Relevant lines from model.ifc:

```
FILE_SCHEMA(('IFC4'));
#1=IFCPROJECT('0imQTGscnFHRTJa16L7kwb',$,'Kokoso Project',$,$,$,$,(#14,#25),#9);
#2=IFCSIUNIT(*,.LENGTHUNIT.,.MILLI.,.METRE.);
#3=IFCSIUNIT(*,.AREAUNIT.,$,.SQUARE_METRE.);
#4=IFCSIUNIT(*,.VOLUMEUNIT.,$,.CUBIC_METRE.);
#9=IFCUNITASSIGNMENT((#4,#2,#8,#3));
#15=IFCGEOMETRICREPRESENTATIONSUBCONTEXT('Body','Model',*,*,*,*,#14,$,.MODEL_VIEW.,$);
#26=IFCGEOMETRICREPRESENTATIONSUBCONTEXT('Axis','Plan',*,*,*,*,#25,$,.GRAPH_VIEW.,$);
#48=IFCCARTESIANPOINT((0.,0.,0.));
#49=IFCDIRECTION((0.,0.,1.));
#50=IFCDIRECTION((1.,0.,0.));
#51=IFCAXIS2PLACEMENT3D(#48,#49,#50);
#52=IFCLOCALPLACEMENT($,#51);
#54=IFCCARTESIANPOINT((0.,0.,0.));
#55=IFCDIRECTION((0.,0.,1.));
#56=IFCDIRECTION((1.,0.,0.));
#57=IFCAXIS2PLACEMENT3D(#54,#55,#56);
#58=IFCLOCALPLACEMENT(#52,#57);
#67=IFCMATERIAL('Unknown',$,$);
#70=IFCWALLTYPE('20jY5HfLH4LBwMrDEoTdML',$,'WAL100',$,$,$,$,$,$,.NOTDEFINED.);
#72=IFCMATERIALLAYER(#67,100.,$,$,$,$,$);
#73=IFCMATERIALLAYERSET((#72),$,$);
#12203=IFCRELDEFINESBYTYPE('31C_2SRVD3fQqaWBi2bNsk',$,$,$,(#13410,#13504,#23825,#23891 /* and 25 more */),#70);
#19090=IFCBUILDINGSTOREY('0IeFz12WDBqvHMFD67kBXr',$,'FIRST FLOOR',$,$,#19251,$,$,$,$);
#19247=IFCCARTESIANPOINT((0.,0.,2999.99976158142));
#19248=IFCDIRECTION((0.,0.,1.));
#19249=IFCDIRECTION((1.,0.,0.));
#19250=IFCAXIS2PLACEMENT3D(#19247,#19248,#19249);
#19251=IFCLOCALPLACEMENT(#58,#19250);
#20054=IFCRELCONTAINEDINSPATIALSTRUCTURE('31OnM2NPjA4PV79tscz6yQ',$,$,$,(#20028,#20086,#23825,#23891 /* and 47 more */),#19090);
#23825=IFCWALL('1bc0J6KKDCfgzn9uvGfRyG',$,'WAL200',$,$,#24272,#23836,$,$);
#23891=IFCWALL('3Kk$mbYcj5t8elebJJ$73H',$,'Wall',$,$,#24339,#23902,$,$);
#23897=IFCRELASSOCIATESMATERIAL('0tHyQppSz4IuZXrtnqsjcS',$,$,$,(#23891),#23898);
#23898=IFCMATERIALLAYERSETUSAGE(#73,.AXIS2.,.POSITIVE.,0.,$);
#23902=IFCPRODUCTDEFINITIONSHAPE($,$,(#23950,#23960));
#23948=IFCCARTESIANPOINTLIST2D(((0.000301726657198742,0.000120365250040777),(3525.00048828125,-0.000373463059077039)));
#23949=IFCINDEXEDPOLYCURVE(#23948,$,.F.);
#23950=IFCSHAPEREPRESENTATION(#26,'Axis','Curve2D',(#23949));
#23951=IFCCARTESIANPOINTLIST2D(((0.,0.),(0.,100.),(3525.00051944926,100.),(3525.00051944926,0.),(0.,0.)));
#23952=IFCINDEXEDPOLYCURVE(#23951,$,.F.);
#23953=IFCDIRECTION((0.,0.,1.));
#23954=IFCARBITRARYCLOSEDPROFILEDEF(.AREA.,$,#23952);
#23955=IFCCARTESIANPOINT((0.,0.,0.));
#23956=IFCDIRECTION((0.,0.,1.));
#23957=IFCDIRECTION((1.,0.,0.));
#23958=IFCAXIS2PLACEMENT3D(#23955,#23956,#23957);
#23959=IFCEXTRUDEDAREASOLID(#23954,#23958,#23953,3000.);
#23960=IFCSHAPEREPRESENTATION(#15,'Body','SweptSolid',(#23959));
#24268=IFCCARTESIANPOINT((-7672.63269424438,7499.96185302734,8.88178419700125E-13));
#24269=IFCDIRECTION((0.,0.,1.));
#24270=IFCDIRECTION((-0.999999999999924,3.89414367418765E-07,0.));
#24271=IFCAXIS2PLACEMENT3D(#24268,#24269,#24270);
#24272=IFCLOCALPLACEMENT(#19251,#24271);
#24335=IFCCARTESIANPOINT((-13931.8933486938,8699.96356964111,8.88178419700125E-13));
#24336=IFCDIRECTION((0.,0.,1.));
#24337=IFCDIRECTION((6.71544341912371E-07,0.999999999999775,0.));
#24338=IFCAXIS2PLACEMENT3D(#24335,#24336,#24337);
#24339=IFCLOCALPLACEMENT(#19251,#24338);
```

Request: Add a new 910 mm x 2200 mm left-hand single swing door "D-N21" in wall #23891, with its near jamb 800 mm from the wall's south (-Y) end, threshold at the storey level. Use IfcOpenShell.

```python
import numpy as np
import ifcopenshell
import ifcopenshell.api.feature
import ifcopenshell.api.geometry
import ifcopenshell.api.root
import ifcopenshell.api.spatial
import ifcopenshell.geom
import ifcopenshell.util.element
import ifcopenshell.util.placement
import ifcopenshell.util.representation
import ifcopenshell.util.shape
import ifcopenshell.util.unit

model = ifcopenshell.open("model.ifc")
unit_scale = ifcopenshell.util.unit.calculate_unit_scale(model)
settings = ifcopenshell.geom.settings()


def volume(element):
    """Net volume in cubic metres, openings subtracted."""
    shape = ifcopenshell.geom.create_shape(settings, element)
    return ifcopenshell.util.shape.get_volume(shape.geometry)


wall = model.by_guid("3Kk$mbYcj5t8elebJJ$73H")
storey = ifcopenshell.util.element.get_container(wall, ifc_class="IfcBuildingStorey")
context = ifcopenshell.util.representation.get_context(model, "Model", "Body", "MODEL_VIEW")
before = volume(wall)

width, height, from_end, sill = 0.91, 2.2, 0.8, 0.0  # metres

# The wall runs along its own X axis, and the end named is its -X end.
wall_shape = ifcopenshell.geom.create_shape(settings, wall)
x, y, z = ifcopenshell.util.shape.get_vertices(wall_shape.geometry).T
start = x.min() + from_end
face, thickness = float(y.min()), float(y.max() - y.min())
wall_matrix = ifcopenshell.util.placement.get_local_placement(wall.ObjectPlacement)
level = ifcopenshell.util.placement.get_local_placement(storey.ObjectPlacement)[2, 3]


def in_wall(x, y):
    """Placement at x, y metres in the wall's axes, at sill height."""
    matrix = wall_matrix.copy()
    matrix[:, 3] = wall_matrix @ np.array([x / unit_scale, y / unit_scale, 0.0, 1.0])
    matrix[2, 3] = level + sill / unit_scale
    return matrix


# Opening: a box that overshoots both wall faces by 50 mm.
opening = ifcopenshell.api.root.create_entity(model, ifc_class="IfcOpeningElement", predefined_type="OPENING")
box = ifcopenshell.api.geometry.add_wall_representation(
    model, context=context, length=width, height=height, thickness=thickness + 0.1
)
ifcopenshell.api.geometry.assign_representation(model, product=opening, representation=box)
ifcopenshell.api.geometry.edit_object_placement(model, product=opening, matrix=in_wall(start, face - 0.05), is_si=False)
ifcopenshell.api.feature.add_feature(model, feature=opening, element=wall)

door = ifcopenshell.api.root.create_entity(model, ifc_class="IfcDoor", name="D-N21", predefined_type="DOOR")
door.OverallWidth, door.OverallHeight = width / unit_scale, height / unit_scale
door.OperationType = "SINGLE_SWING_LEFT"
body = ifcopenshell.api.geometry.add_door_representation(
    model,
    context=context,
    overall_width=door.OverallWidth,
    overall_height=door.OverallHeight,
    operation_type="SINGLE_SWING_LEFT",
    lining_properties={"LiningDepth": thickness / unit_scale, "ThresholdDepth": thickness / unit_scale},
)
ifcopenshell.api.geometry.assign_representation(model, product=door, representation=body)
ifcopenshell.api.spatial.assign_container(model, products=[door], relating_structure=storey)
ifcopenshell.api.feature.add_filling(model, opening=opening, element=door)

# The lining spans the wall, so the door starts at the wall face.
ifcopenshell.api.geometry.edit_object_placement(model, product=door, matrix=in_wall(start, face), is_si=False)

after = volume(wall)

print(f"wall volume {before:.3f} -> {after:.3f} m3")

model.write("model_updated.ifc")
```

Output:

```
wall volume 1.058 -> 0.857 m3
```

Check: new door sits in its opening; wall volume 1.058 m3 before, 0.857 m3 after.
